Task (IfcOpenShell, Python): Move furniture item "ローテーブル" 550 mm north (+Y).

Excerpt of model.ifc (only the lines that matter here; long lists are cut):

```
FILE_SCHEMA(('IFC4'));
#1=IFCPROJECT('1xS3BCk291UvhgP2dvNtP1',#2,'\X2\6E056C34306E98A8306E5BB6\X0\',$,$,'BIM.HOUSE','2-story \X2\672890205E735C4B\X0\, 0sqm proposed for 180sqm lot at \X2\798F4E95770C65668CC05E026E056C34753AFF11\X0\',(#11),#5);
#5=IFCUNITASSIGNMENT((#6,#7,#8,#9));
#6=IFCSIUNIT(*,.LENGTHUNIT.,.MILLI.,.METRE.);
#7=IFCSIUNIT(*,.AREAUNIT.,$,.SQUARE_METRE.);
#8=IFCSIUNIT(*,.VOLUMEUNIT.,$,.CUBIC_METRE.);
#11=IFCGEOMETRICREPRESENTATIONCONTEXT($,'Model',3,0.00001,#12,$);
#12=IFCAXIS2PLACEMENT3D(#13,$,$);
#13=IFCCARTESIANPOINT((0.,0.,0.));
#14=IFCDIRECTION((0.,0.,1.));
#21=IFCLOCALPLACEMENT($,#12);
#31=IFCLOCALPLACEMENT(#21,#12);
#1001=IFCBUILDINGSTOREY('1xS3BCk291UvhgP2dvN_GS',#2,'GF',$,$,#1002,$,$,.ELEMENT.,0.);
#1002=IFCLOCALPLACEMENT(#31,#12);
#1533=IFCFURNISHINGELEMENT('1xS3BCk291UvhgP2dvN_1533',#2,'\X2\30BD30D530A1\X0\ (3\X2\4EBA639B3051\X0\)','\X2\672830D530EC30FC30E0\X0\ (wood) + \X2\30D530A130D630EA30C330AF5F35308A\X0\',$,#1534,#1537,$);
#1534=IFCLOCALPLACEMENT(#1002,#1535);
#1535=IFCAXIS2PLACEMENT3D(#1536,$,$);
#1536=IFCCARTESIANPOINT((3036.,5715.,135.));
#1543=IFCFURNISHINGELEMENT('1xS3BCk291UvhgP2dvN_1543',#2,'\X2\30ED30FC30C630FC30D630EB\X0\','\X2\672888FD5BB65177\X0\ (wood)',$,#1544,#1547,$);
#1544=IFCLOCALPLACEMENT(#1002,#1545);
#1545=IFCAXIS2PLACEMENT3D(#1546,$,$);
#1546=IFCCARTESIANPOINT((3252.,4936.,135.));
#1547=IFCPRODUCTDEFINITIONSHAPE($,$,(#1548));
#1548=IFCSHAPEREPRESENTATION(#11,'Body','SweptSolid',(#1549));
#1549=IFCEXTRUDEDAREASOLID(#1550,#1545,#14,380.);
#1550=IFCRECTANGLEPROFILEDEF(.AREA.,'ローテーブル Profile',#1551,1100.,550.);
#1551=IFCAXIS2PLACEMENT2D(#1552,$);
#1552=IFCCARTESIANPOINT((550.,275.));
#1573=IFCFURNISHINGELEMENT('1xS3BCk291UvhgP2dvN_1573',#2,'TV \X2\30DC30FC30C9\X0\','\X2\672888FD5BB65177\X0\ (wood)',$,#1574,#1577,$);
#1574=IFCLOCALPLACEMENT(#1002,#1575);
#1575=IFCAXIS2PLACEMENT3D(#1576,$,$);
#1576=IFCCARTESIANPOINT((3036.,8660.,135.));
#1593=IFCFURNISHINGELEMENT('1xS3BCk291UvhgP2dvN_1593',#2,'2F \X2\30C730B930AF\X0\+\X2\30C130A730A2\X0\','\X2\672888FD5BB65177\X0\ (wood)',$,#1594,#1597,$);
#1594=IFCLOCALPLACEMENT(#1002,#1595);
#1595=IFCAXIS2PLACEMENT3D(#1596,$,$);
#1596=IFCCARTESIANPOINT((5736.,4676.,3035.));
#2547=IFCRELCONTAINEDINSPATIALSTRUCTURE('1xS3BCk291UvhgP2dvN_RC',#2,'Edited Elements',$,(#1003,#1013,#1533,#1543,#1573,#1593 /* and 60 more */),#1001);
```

```python
import ifcopenshell
import ifcopenshell.api.geometry
import ifcopenshell.util.placement

model = ifcopenshell.open("model.ifc")

item = model.by_guid("1xS3BCk291UvhgP2dvN_1543")
matrix = ifcopenshell.util.placement.get_local_placement(item.ObjectPlacement)
matrix[1, 3] += 550.0
ifcopenshell.api.geometry.edit_object_placement(model, product=item, matrix=matrix, is_si=False)

print(ifcopenshell.util.placement.get_local_placement(item.ObjectPlacement).round(3) + 0.0)

model.write("model_edited.ifc")
```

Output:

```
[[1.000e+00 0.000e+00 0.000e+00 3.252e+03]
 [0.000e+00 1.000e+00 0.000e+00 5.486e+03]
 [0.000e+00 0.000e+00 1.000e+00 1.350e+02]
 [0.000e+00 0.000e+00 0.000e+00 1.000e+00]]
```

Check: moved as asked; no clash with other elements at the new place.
